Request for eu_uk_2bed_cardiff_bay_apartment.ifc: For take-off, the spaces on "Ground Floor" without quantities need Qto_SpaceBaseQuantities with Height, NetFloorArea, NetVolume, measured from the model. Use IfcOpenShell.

First a look at what the model holds.

```python
import ifcopenshell
import ifcopenshell.util.element
import ifcopenshell.util.unit

model = ifcopenshell.open("eu_uk_2bed_cardiff_bay_apartment.ifc")
print(model.schema)
for unit_type in ("LENGTHUNIT", "AREAUNIT", "VOLUMEUNIT"):
    print(unit_type, ifcopenshell.util.unit.calculate_unit_scale(model, unit_type))
storey = next(s for s in model.by_type("IfcBuildingStorey") if s.Name == "Ground Floor")
spaces = [e for e in ifcopenshell.util.element.get_decomposition(storey) if e.is_a("IfcSpace")]
for e in sorted(spaces, key=lambda e: e.id()):
    print(e.id(), e.is_a(), e.Name, list(ifcopenshell.util.element.get_psets(e, qtos_only=True)), sep=" | ")
```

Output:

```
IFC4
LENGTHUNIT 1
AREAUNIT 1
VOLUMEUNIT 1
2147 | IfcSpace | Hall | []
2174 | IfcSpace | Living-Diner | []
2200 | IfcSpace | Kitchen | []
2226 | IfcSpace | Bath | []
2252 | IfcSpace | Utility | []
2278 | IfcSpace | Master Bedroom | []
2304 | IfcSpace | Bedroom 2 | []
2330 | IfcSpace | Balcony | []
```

```python
import ifcopenshell
import ifcopenshell.api.pset
import ifcopenshell.geom
import ifcopenshell.util.element
import ifcopenshell.util.shape
import ifcopenshell.util.unit

model = ifcopenshell.open("eu_uk_2bed_cardiff_bay_apartment.ifc")
unit_scale = ifcopenshell.util.unit.calculate_unit_scale(model)
area_scale = ifcopenshell.util.unit.calculate_unit_scale(model, "AREAUNIT")
volume_scale = ifcopenshell.util.unit.calculate_unit_scale(model, "VOLUMEUNIT")
settings = ifcopenshell.geom.settings()

storey = next(s for s in model.by_type("IfcBuildingStorey") if s.Name == "Ground Floor")
spaces = [e for e in ifcopenshell.util.element.get_decomposition(storey) if e.is_a("IfcSpace")]

for e in sorted(spaces, key=lambda e: e.id()):
    if ifcopenshell.util.element.get_psets(e, qtos_only=True, should_inherit=False):
        continue
    # Geometry comes back in metres, in the element's own axes.
    shape = ifcopenshell.geom.create_shape(settings, e)
    values = {
        "Height": ifcopenshell.util.shape.get_z(shape.geometry) / unit_scale,
        "NetFloorArea": ifcopenshell.util.shape.get_footprint_area(shape.geometry) / area_scale,
        "NetVolume": ifcopenshell.util.shape.get_volume(shape.geometry) / volume_scale,
    }
    qto = ifcopenshell.api.pset.add_qto(model, product=e, name="Qto_SpaceBaseQuantities")
    ifcopenshell.api.pset.edit_qto(model, qto=qto, properties=values)
    print(e.id(), {k: round(v, 3) for k, v in values.items()})

model.write("eu_uk_2bed_cardiff_bay_apartment_edited.ifc")
```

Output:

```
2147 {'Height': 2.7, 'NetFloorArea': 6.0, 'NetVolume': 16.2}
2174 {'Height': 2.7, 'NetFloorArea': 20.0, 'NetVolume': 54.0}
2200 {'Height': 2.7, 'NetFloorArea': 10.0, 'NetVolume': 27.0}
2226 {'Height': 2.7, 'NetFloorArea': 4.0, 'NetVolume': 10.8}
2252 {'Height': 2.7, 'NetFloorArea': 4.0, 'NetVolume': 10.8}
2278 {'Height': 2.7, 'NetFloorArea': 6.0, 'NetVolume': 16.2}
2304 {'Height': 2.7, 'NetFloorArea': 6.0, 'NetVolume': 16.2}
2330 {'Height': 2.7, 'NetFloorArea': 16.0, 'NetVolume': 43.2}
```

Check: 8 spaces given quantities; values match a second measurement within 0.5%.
